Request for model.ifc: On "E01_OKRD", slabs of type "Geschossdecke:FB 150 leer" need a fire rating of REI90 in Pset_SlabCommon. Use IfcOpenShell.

First a look at what the model holds.

```python
import ifcopenshell
import ifcopenshell.util.element

model = ifcopenshell.open("model.ifc")
print(model.schema)
storey = next(s for s in model.by_type("IfcBuildingStorey") if s.Name == "E01_OKRD")
slabs = [e for e in ifcopenshell.util.element.get_decomposition(storey) if e.is_a("IfcSlab")]
seen = {}
for e in slabs:
    element_type = ifcopenshell.util.element.get_type(e)
    key = (element_type.Name if element_type != e and element_type else None, ifcopenshell.util.element.get_pset(e, "Pset_SlabCommon", "FireRating"))
    seen[key] = seen.get(key, 0) + 1
for (name, value), count in sorted(seen.items(), key=str):
    print(count, "x", name, "|", value)
```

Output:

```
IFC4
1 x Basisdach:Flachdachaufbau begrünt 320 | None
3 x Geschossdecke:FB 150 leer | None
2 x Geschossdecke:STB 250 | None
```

```python
import ifcopenshell
import ifcopenshell.api.pset
import ifcopenshell.util.element

model = ifcopenshell.open("model.ifc")

storey = next(s for s in model.by_type("IfcBuildingStorey") if s.Name == "E01_OKRD")
slabs = [e for e in ifcopenshell.util.element.get_decomposition(storey) if e.is_a("IfcSlab")]

count = 0
for e in slabs:
    element_type = ifcopenshell.util.element.get_type(e)
    if element_type in (None, e) or element_type.Name != "Geschossdecke:FB 150 leer":
        continue
    # add_pset returns the element's existing set when there is one.
    pset = ifcopenshell.api.pset.add_pset(model, product=e, name="Pset_SlabCommon")
    ifcopenshell.api.pset.edit_pset(model, pset=pset, properties={"FireRating": "REI90"})
    count += 1

print(count, "slabs updated")

model.write("model_rev.ifc")
```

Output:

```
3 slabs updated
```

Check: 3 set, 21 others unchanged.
